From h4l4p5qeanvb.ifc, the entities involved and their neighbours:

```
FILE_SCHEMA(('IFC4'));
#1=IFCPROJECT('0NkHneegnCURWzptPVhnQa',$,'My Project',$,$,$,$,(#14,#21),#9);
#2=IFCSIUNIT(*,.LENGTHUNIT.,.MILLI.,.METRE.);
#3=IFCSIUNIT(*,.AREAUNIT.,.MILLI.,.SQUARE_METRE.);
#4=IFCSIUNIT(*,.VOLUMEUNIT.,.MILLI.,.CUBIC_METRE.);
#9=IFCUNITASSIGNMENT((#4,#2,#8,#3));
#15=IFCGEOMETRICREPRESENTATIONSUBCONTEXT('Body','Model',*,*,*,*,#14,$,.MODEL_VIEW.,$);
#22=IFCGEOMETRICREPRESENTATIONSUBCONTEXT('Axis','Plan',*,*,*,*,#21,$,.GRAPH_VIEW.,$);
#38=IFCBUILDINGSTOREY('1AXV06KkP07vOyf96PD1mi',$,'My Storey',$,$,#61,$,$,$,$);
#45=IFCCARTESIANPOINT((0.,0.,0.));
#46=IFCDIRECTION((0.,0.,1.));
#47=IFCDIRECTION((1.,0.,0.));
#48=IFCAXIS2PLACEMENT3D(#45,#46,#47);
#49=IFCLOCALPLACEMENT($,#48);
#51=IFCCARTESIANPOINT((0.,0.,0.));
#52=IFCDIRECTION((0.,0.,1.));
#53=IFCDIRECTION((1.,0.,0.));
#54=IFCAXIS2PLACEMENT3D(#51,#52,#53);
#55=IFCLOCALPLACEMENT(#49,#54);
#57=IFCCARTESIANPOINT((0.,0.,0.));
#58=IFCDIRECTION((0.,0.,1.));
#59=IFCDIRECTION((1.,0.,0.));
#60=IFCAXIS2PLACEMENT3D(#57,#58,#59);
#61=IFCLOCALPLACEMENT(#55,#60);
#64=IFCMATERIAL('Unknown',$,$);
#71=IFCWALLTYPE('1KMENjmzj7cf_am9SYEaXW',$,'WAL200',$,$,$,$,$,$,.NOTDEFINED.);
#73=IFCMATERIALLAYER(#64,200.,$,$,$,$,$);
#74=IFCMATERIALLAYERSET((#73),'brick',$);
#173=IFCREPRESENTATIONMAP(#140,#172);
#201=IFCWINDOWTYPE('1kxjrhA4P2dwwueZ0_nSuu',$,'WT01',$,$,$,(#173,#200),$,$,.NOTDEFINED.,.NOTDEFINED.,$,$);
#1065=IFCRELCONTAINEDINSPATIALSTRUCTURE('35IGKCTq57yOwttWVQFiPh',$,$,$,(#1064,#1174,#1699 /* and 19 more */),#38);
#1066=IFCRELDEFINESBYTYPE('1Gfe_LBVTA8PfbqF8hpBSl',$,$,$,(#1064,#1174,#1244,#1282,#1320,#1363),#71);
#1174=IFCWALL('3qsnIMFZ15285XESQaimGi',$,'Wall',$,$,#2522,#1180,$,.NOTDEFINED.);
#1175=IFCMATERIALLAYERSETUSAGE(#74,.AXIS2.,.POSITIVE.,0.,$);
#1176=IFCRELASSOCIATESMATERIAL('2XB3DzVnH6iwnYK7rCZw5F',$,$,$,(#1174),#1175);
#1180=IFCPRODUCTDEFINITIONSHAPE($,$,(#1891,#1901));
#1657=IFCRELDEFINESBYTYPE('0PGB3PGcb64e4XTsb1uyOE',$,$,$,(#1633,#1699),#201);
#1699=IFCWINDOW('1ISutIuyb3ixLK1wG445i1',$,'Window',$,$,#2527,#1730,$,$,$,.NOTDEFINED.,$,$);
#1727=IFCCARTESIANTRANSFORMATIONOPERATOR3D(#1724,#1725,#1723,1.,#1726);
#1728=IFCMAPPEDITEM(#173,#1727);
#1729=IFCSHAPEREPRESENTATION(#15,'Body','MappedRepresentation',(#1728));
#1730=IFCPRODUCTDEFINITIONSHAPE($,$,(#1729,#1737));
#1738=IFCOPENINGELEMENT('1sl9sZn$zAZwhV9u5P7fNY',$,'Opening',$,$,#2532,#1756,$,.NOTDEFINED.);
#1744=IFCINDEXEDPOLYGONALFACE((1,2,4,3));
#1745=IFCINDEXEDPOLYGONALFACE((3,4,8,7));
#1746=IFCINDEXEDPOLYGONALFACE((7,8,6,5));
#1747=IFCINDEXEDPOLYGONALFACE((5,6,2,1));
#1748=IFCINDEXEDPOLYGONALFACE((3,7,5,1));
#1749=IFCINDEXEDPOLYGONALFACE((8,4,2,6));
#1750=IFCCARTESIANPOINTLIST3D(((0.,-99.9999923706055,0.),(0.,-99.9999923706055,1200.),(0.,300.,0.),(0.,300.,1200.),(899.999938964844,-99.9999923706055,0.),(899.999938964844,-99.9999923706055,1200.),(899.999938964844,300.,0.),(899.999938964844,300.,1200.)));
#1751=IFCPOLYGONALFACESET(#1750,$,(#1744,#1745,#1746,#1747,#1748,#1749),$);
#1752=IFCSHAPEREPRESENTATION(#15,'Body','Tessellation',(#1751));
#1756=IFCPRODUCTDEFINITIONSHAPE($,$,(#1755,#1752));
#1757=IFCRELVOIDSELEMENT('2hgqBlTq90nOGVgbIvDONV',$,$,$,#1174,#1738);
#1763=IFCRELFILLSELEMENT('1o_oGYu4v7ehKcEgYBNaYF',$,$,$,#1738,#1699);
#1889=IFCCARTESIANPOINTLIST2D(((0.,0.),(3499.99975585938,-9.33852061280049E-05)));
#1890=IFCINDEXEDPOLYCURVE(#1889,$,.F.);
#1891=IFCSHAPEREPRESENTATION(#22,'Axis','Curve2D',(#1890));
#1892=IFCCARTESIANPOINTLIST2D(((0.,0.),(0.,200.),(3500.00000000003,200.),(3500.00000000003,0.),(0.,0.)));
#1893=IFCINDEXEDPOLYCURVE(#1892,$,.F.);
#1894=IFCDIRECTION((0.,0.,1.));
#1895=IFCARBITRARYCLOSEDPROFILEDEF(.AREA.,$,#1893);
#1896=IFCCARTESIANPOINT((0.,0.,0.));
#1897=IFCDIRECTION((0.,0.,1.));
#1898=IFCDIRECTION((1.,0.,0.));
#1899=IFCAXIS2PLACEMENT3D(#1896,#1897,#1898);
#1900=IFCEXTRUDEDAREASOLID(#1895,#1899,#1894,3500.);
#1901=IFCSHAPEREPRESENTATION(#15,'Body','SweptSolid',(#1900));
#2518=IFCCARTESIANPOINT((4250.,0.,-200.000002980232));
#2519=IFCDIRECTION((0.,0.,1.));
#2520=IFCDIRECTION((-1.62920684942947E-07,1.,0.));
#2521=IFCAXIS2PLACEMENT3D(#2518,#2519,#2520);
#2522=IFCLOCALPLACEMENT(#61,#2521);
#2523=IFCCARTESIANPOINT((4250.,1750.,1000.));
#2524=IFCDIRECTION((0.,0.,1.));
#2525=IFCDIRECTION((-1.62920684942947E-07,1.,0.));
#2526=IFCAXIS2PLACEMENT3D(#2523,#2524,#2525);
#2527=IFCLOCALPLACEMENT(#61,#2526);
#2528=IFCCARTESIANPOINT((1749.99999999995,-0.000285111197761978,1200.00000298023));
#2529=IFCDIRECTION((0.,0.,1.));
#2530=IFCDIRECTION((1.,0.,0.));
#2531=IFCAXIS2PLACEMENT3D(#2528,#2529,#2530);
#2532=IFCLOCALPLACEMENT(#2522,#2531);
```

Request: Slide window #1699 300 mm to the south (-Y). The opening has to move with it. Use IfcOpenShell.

```python
import ifcopenshell
import ifcopenshell.api.geometry
import ifcopenshell.util.placement
import ifcopenshell.util.unit

model = ifcopenshell.open("h4l4p5qeanvb.ifc")
unit_scale = ifcopenshell.util.unit.calculate_unit_scale(model)

window = model.by_id(1699)
opening = window.FillsVoids[0].RelatingOpeningElement
wall = opening.VoidsElements[0].RelatingBuildingElement

wall_matrix = ifcopenshell.util.placement.get_local_placement(wall.ObjectPlacement)
shift = wall_matrix[:3, 0] * -0.3 / unit_scale
before = ifcopenshell.util.placement.get_local_placement(window.ObjectPlacement)[:3, 3].copy()

# The window is not placed relative to its opening, so move both.
for product in (opening, window):
    matrix = ifcopenshell.util.placement.get_local_placement(product.ObjectPlacement)
    matrix[:3, 3] += shift
    ifcopenshell.api.geometry.edit_object_placement(model, product=product, matrix=matrix, is_si=False)

after = ifcopenshell.util.placement.get_local_placement(window.ObjectPlacement)[:3, 3]
print("window moved by", (after - before).round(3) + 0.0)

model.write("h4l4p5qeanvb_edited.ifc")
```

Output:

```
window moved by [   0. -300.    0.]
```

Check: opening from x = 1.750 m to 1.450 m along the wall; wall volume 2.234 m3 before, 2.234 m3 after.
